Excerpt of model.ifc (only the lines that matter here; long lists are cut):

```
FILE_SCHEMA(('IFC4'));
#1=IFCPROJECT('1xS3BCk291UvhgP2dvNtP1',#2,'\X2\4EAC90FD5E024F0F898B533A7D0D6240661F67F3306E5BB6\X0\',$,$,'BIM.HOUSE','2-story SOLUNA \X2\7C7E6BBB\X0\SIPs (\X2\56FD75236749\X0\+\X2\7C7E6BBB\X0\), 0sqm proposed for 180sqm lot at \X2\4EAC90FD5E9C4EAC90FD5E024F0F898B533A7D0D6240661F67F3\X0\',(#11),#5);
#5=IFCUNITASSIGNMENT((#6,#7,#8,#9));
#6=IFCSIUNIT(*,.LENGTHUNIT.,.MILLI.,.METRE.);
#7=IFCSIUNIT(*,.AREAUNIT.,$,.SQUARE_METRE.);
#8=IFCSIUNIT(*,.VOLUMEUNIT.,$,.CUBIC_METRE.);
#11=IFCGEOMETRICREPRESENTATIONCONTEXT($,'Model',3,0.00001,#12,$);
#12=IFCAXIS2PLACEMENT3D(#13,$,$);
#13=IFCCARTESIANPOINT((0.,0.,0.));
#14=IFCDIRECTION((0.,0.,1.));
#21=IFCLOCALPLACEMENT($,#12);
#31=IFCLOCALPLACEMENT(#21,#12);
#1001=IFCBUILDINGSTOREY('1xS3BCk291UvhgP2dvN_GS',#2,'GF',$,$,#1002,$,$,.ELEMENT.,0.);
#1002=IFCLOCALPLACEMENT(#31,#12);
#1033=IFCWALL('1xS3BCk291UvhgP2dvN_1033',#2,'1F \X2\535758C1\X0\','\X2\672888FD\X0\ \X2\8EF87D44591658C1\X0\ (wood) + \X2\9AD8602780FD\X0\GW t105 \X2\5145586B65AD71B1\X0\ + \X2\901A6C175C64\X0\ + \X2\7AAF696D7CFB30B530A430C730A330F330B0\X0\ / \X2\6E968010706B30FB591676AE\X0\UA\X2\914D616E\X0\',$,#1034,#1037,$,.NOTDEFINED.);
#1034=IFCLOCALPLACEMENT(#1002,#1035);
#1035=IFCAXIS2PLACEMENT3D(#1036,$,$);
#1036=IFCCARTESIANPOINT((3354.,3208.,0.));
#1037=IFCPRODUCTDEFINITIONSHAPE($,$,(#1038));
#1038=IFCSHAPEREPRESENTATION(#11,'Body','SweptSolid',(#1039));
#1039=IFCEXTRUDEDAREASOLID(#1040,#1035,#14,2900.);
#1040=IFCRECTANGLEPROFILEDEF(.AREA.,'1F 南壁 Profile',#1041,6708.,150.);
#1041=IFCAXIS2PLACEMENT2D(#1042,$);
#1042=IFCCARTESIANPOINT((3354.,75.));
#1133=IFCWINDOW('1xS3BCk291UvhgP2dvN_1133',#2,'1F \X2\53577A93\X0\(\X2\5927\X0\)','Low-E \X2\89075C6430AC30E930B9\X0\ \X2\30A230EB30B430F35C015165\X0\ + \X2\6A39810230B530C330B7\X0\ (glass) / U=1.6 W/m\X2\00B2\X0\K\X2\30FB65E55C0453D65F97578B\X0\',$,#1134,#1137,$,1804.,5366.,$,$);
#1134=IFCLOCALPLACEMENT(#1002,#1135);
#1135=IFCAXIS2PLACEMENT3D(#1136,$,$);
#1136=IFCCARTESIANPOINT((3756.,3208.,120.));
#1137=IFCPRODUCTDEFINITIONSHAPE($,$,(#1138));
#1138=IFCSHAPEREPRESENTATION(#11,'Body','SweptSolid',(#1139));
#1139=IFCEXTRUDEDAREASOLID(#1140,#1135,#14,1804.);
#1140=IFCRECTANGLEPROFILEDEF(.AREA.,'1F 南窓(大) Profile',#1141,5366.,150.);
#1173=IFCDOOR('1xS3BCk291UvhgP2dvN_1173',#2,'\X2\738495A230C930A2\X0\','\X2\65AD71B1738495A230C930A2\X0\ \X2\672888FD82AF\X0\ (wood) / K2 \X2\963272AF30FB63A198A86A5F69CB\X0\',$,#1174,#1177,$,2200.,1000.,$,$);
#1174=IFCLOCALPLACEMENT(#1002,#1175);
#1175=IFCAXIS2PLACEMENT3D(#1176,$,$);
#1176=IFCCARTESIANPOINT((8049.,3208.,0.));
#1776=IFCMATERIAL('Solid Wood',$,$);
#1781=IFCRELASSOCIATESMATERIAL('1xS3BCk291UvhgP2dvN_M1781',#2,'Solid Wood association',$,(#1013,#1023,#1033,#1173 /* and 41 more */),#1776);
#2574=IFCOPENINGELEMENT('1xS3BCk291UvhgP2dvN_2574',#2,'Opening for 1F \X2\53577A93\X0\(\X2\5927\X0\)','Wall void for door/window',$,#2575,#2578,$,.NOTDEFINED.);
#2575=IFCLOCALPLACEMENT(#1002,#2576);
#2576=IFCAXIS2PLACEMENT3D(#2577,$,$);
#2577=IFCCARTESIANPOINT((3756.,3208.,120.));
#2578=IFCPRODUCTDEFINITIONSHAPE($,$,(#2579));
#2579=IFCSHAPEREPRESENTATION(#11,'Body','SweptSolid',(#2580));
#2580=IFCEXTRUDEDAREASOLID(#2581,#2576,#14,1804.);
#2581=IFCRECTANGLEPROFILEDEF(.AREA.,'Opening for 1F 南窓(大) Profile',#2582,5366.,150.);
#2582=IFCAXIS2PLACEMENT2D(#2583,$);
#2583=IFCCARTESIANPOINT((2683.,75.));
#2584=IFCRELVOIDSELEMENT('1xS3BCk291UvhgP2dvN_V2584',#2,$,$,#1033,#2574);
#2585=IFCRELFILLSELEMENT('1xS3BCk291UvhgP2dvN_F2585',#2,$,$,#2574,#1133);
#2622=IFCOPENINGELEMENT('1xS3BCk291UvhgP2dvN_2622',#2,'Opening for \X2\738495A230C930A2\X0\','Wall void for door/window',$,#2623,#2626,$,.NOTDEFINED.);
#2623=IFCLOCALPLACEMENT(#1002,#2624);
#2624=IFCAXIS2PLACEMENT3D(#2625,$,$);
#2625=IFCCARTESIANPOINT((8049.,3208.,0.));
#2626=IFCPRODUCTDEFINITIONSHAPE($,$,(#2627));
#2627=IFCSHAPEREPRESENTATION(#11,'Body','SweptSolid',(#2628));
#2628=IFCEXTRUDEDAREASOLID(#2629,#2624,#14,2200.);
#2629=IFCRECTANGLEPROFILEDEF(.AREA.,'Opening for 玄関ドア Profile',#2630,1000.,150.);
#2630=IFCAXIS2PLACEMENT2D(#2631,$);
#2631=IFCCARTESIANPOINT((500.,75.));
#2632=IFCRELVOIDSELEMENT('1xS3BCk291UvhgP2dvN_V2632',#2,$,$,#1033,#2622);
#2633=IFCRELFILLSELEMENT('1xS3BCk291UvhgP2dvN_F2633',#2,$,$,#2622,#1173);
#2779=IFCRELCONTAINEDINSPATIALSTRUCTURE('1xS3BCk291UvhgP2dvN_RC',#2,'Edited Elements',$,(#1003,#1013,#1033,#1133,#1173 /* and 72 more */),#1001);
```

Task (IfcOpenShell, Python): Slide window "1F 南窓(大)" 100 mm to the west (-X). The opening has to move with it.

```python
import ifcopenshell
import ifcopenshell.api.geometry
import ifcopenshell.util.placement
import ifcopenshell.util.unit

model = ifcopenshell.open("model.ifc")
unit_scale = ifcopenshell.util.unit.calculate_unit_scale(model)

window = model.by_guid("1xS3BCk291UvhgP2dvN_1133")
opening = window.FillsVoids[0].RelatingOpeningElement
wall = opening.VoidsElements[0].RelatingBuildingElement

wall_matrix = ifcopenshell.util.placement.get_local_placement(wall.ObjectPlacement)
shift = wall_matrix[:3, 0] * -0.1 / unit_scale
before = ifcopenshell.util.placement.get_local_placement(window.ObjectPlacement)[:3, 3].copy()

# The window is not placed relative to its opening, so move both.
for product in (opening, window):
    matrix = ifcopenshell.util.placement.get_local_placement(product.ObjectPlacement)
    matrix[:3, 3] += shift
    ifcopenshell.api.geometry.edit_object_placement(model, product=product, matrix=matrix, is_si=False)

after = ifcopenshell.util.placement.get_local_placement(window.ObjectPlacement)[:3, 3]
print("window moved by", (after - before).round(3) + 0.0)

model.write("model_rev.ifc")
```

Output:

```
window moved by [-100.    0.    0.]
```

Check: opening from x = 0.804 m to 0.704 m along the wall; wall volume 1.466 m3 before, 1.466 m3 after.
